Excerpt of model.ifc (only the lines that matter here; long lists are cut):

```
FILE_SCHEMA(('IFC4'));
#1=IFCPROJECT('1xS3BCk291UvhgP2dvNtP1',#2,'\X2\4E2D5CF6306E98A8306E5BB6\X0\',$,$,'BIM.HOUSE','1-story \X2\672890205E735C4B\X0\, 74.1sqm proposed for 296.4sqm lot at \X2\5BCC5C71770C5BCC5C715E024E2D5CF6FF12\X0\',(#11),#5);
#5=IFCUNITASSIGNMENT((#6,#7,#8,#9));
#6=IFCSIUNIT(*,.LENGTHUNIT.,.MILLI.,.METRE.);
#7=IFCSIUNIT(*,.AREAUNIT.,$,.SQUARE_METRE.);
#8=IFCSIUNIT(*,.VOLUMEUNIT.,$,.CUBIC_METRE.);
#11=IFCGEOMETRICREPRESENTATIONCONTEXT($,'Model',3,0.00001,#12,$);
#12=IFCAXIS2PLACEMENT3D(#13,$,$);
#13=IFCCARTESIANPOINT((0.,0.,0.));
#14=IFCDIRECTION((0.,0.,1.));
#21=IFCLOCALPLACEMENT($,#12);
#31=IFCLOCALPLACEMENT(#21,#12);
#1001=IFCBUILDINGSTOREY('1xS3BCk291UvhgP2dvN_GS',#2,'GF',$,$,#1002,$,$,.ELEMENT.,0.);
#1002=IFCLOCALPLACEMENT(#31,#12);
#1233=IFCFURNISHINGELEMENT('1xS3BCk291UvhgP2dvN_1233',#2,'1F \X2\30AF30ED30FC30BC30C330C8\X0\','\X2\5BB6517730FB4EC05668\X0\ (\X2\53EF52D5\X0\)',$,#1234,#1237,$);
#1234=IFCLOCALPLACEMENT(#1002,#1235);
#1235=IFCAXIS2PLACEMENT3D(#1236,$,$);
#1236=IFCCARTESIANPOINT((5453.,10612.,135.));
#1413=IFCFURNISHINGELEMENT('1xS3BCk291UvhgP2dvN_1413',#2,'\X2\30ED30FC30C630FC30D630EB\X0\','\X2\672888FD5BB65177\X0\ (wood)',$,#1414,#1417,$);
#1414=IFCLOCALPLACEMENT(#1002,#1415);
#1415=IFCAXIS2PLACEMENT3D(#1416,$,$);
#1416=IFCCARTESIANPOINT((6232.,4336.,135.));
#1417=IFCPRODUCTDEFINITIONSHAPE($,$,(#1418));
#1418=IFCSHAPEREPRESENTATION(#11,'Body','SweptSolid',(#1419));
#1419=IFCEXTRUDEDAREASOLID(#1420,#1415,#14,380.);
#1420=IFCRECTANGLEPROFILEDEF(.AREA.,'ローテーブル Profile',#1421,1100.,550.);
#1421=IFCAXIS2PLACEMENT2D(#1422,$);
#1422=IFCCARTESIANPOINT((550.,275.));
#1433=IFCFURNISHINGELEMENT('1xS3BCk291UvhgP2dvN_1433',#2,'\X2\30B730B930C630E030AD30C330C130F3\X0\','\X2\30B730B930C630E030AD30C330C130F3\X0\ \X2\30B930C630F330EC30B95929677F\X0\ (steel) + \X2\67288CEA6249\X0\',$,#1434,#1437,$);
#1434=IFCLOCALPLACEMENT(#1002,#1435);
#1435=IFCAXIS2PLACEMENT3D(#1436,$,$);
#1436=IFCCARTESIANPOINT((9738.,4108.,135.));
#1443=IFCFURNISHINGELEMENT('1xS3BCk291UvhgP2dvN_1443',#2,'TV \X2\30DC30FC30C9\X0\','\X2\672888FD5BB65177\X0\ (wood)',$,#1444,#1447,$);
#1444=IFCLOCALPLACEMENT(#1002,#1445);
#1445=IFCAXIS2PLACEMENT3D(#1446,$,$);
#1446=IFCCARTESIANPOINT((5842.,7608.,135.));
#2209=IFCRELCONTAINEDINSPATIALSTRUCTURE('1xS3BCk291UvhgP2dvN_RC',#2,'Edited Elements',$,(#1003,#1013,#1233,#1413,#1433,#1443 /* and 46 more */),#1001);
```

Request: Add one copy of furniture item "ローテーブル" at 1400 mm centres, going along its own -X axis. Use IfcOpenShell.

```python
import ifcopenshell
import ifcopenshell.api.geometry
import ifcopenshell.api.root
import ifcopenshell.util.element
import ifcopenshell.util.placement

model = ifcopenshell.open("model.ifc")


def reuse_history(source, copy):
    """copy_class also copies each property set's owner history, people and application; keep the originals."""
    for rel in copy.IsDefinedBy:
        if rel.is_a("IfcRelDefinesByProperties") and (history := rel.RelatingPropertyDefinition.OwnerHistory):
            rel.RelatingPropertyDefinition.OwnerHistory = source.OwnerHistory
            ifcopenshell.util.element.remove_deep2(model, history)


source = model.by_guid("1xS3BCk291UvhgP2dvN_1413")
base = ifcopenshell.util.placement.get_local_placement(source.ObjectPlacement)
step = -base[:3, 0] * 1400.0

for i in range(1, 2):
    copy = ifcopenshell.api.root.copy_class(model, product=source)
    copy.Representation = ifcopenshell.util.element.copy_deep(
        model, source.Representation, exclude=["IfcGeometricRepresentationContext", "IfcRepresentationMap"]
    )
    reuse_history(source, copy)
    matrix = base.copy()
    matrix[:3, 3] += i * step
    print("added at", matrix[:3, 3].round(3) + 0.0)
    ifcopenshell.api.geometry.edit_object_placement(model, product=copy, matrix=matrix, is_si=False)

model.write("model_rev.ifc")
```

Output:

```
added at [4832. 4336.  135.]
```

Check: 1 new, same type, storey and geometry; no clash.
